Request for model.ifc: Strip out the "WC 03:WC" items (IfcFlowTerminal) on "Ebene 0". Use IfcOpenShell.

First a look at what the model holds.

```python
import ifcopenshell
import ifcopenshell.util.element

model = ifcopenshell.open("model.ifc")
print(model.schema)
storey = next(s for s in model.by_type("IfcBuildingStorey") if s.Name == "Ebene 0")
terminals = [e for e in ifcopenshell.util.element.get_decomposition(storey) if e.is_a("IfcFlowTerminal")]
seen = {}
for e in terminals:
    element_type = ifcopenshell.util.element.get_type(e)
    name = element_type.Name if element_type not in (None, e) else None
    seen[name] = seen.get(name, 0) + 1
for name, count in sorted(seen.items(), key=str):
    print(count, "x", name)
```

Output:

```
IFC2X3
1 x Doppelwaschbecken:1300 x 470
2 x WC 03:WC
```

```python
import ifcopenshell
import ifcopenshell.api.root
import ifcopenshell.util.element

model = ifcopenshell.open("model.ifc")

storey = next(s for s in model.by_type("IfcBuildingStorey") if s.Name == "Ebene 0")
terminals = [e for e in ifcopenshell.util.element.get_decomposition(storey) if e.is_a("IfcFlowTerminal")]
targets = [e for e in terminals if (t := ifcopenshell.util.element.get_type(e)) not in (None, e) and t.Name == "WC 03:WC"]

for e in targets:
    ifcopenshell.api.root.remove_product(model, product=e)
print(len(targets), "removed")

model.write("model_v2.ifc")
```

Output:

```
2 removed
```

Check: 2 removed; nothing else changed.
